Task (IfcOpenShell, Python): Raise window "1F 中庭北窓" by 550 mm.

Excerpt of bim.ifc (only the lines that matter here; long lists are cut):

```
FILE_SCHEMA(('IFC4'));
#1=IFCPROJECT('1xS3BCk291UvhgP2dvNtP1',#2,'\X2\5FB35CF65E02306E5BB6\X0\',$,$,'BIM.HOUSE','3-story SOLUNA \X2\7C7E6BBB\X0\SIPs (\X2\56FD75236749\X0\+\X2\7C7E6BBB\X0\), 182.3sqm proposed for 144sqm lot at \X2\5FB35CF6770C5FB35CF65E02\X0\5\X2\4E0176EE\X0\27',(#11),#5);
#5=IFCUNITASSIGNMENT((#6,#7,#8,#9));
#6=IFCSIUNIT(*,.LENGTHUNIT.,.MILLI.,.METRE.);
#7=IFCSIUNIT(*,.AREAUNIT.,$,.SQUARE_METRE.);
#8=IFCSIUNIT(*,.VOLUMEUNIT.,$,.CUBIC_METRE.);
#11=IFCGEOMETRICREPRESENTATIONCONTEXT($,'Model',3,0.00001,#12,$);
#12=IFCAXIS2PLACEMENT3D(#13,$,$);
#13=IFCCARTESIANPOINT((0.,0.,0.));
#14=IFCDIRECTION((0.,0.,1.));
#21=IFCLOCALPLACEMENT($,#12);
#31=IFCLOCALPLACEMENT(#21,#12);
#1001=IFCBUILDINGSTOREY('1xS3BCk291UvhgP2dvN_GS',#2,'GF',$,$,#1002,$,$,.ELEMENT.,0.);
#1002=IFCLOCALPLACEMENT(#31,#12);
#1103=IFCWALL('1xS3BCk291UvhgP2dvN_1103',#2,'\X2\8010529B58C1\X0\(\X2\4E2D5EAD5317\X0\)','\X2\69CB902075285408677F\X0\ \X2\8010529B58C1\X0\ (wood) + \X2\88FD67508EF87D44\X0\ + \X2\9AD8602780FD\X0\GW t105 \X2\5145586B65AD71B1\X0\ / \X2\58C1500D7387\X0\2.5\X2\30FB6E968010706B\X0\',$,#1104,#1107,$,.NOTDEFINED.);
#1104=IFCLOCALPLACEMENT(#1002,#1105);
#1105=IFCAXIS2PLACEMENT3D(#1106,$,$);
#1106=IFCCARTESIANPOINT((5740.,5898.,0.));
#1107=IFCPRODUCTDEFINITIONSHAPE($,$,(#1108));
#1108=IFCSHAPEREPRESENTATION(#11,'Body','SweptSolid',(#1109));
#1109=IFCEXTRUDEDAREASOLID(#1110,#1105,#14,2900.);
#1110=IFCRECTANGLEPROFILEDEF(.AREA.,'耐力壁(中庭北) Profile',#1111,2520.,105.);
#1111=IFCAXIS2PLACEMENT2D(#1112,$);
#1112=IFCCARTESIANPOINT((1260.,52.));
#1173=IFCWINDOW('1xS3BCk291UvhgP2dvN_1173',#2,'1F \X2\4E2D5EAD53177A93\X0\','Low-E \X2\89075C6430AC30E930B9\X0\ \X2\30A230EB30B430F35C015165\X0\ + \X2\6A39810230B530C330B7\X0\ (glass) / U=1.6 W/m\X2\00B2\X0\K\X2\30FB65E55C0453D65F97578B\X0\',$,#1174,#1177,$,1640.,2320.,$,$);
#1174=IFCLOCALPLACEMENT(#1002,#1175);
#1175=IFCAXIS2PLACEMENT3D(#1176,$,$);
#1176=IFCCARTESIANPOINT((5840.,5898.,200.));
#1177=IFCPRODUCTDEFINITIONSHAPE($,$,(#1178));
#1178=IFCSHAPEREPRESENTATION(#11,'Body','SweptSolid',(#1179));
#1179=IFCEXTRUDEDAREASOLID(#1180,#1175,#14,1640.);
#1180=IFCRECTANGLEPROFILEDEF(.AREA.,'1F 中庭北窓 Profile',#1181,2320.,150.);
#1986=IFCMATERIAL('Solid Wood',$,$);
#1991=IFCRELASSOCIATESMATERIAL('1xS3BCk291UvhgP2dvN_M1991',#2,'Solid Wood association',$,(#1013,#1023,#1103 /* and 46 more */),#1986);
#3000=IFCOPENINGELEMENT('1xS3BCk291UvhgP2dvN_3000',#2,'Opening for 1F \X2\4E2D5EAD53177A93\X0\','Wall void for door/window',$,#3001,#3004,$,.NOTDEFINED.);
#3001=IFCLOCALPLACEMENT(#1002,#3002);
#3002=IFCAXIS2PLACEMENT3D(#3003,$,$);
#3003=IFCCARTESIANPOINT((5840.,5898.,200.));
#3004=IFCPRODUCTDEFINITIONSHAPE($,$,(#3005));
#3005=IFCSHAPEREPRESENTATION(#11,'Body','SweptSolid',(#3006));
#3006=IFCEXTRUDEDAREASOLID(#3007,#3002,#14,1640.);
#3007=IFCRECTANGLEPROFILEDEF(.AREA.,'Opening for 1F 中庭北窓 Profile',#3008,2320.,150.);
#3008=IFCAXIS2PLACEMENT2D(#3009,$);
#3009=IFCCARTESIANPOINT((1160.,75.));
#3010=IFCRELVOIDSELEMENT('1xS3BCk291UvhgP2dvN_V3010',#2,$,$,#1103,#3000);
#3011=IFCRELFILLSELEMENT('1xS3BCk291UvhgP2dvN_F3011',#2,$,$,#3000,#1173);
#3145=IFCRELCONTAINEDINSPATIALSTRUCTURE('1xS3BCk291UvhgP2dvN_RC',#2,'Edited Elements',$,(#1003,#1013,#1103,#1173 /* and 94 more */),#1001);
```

```python
import numpy as np
import ifcopenshell
import ifcopenshell.api.geometry
import ifcopenshell.util.placement
import ifcopenshell.util.unit

model = ifcopenshell.open("bim.ifc")
unit_scale = ifcopenshell.util.unit.calculate_unit_scale(model)

window = model.by_guid("1xS3BCk291UvhgP2dvN_1173")
opening = window.FillsVoids[0].RelatingOpeningElement
dz = 550.0

shift = np.array([0.0, 0.0, dz])
# The window is not placed relative to its opening, so move both.
for product in (opening, window):
    matrix = ifcopenshell.util.placement.get_local_placement(product.ObjectPlacement)
    matrix[:3, 3] += shift
    ifcopenshell.api.geometry.edit_object_placement(model, product=product, matrix=matrix, is_si=False)

print(f"moved by {dz * unit_scale:+.3f} m")

model.write("bim-out.ifc")
```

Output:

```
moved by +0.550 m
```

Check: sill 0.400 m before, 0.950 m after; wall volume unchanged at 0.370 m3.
